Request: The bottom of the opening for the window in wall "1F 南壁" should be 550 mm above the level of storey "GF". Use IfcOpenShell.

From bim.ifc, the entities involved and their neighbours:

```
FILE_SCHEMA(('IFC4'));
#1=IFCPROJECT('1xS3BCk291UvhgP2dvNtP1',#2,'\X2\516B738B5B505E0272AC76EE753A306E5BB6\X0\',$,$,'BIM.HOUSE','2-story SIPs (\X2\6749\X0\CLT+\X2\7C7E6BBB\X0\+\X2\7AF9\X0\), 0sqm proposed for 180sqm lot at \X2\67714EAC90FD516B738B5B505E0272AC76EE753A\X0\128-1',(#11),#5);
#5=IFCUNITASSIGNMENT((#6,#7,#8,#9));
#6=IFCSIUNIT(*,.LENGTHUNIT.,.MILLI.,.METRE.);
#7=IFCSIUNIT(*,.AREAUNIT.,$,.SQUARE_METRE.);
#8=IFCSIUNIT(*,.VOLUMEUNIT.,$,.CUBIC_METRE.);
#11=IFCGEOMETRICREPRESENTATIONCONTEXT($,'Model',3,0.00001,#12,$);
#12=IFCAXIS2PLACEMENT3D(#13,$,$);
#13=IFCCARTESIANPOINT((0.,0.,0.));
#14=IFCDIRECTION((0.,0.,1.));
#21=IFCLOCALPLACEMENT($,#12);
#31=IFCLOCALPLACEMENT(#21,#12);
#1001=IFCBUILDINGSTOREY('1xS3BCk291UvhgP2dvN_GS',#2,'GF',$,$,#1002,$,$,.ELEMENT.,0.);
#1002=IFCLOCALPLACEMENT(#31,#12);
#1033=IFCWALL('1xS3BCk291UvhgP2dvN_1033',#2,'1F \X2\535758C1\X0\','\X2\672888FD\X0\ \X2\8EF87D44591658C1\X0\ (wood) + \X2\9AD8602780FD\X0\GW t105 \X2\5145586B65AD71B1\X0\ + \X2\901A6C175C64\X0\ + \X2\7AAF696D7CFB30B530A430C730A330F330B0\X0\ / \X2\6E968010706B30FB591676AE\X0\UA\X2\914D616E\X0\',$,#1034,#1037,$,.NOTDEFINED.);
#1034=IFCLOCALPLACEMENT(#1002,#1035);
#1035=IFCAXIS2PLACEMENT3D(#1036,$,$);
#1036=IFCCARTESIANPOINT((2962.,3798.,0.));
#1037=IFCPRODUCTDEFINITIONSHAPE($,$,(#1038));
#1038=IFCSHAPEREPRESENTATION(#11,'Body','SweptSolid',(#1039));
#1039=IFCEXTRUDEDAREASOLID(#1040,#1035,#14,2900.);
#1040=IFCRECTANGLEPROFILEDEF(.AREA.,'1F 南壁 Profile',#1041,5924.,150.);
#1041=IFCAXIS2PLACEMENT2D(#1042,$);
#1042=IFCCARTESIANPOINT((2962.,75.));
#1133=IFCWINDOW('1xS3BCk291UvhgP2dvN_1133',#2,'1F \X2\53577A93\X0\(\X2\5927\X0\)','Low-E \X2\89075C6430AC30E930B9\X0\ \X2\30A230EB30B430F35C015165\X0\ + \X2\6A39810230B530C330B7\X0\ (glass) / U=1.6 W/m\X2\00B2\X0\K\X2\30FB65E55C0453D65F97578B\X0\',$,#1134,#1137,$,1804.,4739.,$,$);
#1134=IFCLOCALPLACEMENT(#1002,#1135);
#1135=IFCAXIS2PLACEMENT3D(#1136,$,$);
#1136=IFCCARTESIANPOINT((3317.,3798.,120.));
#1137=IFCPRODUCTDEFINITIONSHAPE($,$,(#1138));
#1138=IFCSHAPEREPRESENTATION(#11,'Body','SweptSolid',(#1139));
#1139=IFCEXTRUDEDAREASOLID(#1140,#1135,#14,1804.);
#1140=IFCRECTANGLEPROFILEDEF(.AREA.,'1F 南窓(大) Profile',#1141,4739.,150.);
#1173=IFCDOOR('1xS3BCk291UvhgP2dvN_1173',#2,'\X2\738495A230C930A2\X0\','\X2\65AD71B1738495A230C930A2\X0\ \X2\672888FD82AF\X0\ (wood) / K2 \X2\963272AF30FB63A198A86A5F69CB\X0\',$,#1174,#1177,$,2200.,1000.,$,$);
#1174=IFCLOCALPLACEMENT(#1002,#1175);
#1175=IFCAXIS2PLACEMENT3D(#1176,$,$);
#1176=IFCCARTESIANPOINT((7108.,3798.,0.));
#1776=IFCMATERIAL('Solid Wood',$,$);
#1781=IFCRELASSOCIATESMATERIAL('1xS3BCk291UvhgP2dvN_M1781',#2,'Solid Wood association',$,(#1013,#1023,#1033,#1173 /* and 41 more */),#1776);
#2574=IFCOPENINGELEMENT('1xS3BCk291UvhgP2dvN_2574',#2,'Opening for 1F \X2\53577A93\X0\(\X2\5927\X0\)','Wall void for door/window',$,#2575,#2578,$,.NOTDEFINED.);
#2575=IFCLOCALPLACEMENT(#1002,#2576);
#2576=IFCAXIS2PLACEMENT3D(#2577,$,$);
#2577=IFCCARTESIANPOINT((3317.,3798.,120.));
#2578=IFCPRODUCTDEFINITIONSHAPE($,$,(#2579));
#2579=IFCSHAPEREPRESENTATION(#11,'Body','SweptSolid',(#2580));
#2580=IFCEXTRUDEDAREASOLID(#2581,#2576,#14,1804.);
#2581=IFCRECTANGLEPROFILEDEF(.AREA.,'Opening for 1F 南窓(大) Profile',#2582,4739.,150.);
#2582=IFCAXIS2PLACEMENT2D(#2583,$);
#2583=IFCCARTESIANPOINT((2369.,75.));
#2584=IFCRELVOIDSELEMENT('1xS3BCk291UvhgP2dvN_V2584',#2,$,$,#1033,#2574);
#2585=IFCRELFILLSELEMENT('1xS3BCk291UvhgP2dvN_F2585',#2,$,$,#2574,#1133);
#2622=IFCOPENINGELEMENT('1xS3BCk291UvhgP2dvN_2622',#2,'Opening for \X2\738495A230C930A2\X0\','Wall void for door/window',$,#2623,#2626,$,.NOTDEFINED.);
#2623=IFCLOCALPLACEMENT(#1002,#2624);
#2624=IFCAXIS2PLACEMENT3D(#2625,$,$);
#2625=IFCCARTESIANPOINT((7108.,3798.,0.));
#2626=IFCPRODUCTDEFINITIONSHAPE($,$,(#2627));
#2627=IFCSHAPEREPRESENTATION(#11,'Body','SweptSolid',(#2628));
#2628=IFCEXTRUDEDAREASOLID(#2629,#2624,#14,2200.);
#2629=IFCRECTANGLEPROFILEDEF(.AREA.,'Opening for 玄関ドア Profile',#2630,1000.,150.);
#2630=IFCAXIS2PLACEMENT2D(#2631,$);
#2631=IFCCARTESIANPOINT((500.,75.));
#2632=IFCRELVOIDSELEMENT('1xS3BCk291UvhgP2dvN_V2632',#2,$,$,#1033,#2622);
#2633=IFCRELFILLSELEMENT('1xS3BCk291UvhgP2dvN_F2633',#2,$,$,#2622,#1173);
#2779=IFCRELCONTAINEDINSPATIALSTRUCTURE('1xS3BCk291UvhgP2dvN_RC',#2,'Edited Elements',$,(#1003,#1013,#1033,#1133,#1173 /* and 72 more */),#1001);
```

```python
import numpy as np
import ifcopenshell
import ifcopenshell.api.geometry
import ifcopenshell.geom
import ifcopenshell.util.element
import ifcopenshell.util.placement
import ifcopenshell.util.shape
import ifcopenshell.util.unit

model = ifcopenshell.open("bim.ifc")
unit_scale = ifcopenshell.util.unit.calculate_unit_scale(model)

window = model.by_id(1133)
opening = window.FillsVoids[0].RelatingOpeningElement
storey = ifcopenshell.util.element.get_container(window, ifc_class="IfcBuildingStorey")
level = ifcopenshell.util.placement.get_local_placement(storey.ObjectPlacement)[2, 3]

# The opening's origin need not be at the sill, so measure its lowest point.
shape = ifcopenshell.geom.create_shape(ifcopenshell.geom.settings(), opening)
bottom = ifcopenshell.util.shape.get_shape_bottom_elevation(shape, shape.geometry) / unit_scale
dz = level + 550.0 - bottom

shift = np.array([0.0, 0.0, dz])
# The window is not placed relative to its opening, so move both.
for product in (opening, window):
    matrix = ifcopenshell.util.placement.get_local_placement(product.ObjectPlacement)
    matrix[:3, 3] += shift
    ifcopenshell.api.geometry.edit_object_placement(model, product=product, matrix=matrix, is_si=False)

print(f"moved by {dz * unit_scale:+.3f} m")

model.write("bim-out.ifc")
```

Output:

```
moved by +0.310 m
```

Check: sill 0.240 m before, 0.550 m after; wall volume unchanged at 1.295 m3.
